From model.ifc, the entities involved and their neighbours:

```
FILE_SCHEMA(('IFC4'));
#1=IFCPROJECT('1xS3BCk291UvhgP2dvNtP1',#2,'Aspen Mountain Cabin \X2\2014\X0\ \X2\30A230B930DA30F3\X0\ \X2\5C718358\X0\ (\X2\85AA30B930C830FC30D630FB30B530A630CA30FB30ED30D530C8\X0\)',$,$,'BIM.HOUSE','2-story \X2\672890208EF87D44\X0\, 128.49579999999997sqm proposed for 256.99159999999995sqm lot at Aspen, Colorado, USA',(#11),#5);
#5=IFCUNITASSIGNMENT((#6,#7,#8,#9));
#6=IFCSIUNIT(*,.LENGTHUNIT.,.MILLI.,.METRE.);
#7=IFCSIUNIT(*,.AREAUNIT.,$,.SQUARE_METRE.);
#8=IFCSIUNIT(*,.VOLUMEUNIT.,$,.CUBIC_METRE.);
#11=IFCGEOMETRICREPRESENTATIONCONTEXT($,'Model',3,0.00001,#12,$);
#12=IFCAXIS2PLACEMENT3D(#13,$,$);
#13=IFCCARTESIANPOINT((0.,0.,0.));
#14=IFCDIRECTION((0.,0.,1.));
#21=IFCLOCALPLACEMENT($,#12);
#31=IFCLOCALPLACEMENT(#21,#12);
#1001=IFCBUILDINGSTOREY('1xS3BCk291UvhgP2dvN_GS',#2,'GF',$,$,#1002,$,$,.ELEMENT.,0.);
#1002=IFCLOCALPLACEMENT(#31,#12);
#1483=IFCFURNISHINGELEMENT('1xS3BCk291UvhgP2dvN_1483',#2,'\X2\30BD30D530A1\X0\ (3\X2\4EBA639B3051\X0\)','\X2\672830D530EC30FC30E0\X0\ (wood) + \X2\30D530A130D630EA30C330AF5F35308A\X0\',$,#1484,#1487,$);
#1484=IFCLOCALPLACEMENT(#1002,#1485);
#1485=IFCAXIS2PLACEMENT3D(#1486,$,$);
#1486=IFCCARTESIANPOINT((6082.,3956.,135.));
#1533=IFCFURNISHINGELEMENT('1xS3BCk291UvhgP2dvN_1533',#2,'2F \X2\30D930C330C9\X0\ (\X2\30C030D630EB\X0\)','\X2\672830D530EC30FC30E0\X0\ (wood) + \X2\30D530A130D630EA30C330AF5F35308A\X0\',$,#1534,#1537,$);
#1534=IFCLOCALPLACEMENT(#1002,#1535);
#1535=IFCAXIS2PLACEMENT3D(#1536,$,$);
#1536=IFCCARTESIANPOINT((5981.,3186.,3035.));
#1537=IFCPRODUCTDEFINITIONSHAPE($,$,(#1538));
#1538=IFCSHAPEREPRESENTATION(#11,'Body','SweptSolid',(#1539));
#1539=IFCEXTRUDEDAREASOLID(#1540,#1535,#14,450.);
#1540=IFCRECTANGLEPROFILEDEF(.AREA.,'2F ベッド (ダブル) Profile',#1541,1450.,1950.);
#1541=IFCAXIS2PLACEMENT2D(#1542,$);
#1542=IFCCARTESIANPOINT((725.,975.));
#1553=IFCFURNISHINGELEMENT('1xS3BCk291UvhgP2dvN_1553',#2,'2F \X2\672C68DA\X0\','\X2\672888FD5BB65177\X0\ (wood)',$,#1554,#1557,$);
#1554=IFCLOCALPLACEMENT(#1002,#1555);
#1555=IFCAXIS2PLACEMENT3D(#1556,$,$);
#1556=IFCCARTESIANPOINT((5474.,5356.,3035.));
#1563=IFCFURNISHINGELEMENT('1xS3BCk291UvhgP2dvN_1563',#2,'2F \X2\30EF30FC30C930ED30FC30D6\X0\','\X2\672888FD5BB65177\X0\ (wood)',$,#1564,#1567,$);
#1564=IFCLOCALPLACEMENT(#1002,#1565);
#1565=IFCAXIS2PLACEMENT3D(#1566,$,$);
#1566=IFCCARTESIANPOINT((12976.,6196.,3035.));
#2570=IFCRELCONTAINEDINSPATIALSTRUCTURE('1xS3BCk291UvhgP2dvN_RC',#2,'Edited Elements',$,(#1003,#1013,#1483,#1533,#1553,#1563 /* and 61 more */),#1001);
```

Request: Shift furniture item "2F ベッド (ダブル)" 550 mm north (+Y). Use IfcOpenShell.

```python
import ifcopenshell
import ifcopenshell.api.geometry
import ifcopenshell.util.placement

model = ifcopenshell.open("model.ifc")

item = model.by_guid("1xS3BCk291UvhgP2dvN_1533")
matrix = ifcopenshell.util.placement.get_local_placement(item.ObjectPlacement)
matrix[1, 3] += 550.0
ifcopenshell.api.geometry.edit_object_placement(model, product=item, matrix=matrix, is_si=False)

print(ifcopenshell.util.placement.get_local_placement(item.ObjectPlacement).round(3) + 0.0)

model.write("model_edited.ifc")
```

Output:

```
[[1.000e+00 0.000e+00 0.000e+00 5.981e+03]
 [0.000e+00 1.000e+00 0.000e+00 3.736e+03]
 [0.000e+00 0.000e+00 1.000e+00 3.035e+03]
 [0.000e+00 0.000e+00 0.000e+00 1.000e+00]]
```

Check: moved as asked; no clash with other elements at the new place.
